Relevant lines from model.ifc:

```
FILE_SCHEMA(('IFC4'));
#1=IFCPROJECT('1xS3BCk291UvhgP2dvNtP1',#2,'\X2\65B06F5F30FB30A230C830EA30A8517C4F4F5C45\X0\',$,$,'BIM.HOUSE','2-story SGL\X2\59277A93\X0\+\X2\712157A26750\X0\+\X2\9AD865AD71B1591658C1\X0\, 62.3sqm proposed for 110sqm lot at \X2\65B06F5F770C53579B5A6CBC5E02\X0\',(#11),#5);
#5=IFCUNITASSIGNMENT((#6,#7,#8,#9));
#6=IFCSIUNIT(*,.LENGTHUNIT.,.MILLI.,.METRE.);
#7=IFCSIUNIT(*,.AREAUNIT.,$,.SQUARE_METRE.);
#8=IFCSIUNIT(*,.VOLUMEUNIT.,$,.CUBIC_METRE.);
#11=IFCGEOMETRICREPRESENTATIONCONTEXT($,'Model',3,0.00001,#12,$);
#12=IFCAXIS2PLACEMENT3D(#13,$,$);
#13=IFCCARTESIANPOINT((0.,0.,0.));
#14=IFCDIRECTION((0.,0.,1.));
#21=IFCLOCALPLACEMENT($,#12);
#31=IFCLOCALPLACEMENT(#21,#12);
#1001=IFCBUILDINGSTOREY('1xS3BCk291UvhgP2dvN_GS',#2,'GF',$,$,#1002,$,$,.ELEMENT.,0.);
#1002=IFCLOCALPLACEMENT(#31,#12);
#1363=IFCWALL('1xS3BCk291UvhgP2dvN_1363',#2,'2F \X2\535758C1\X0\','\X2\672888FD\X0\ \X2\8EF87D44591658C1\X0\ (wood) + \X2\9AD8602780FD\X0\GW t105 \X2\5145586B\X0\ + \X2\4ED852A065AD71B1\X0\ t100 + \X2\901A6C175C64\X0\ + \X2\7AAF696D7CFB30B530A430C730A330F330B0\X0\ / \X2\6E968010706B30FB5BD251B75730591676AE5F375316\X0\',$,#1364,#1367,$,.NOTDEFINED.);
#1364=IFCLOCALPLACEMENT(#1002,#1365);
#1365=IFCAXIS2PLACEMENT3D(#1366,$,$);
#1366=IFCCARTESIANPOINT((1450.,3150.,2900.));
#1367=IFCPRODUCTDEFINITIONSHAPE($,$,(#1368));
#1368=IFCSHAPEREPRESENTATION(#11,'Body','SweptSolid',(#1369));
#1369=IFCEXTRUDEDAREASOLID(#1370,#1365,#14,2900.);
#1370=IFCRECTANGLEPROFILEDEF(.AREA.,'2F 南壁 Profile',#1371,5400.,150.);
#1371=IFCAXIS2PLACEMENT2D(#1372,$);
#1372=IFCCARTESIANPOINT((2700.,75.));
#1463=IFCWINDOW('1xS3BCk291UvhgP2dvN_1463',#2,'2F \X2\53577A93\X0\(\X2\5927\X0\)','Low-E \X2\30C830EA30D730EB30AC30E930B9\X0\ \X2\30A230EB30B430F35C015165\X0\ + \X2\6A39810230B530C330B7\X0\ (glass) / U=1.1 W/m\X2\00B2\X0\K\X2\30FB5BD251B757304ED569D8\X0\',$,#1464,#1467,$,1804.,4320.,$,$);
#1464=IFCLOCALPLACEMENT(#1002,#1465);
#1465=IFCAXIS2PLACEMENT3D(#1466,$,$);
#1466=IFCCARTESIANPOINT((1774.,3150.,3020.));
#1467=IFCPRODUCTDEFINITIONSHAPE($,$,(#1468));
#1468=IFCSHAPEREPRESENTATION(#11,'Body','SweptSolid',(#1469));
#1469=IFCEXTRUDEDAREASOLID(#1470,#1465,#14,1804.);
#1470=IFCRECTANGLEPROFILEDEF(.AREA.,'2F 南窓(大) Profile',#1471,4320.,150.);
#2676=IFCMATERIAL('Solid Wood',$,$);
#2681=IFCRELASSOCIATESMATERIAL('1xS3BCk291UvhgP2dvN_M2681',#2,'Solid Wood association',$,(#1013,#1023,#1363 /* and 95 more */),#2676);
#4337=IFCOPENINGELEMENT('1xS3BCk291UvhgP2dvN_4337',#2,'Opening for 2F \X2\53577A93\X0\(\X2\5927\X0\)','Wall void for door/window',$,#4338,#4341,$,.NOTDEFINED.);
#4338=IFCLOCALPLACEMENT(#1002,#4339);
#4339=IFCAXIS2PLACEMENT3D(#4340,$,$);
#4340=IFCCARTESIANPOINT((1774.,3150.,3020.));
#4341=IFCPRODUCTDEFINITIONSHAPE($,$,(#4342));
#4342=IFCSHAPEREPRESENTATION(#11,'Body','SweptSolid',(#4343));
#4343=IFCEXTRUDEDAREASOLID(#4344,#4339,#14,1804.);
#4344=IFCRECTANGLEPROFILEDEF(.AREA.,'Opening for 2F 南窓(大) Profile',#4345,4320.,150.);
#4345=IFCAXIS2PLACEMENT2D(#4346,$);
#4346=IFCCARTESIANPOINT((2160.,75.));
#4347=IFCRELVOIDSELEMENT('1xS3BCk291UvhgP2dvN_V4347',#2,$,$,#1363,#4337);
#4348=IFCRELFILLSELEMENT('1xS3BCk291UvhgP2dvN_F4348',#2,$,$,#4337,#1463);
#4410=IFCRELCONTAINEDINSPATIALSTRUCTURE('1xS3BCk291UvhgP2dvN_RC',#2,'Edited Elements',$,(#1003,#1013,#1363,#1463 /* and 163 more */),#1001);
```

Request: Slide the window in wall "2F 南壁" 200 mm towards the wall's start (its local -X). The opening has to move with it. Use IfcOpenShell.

```python
import ifcopenshell
import ifcopenshell.api.geometry
import ifcopenshell.util.placement
import ifcopenshell.util.unit

model = ifcopenshell.open("model.ifc")
unit_scale = ifcopenshell.util.unit.calculate_unit_scale(model)

window = model.by_guid("1xS3BCk291UvhgP2dvN_1463")
opening = window.FillsVoids[0].RelatingOpeningElement
wall = opening.VoidsElements[0].RelatingBuildingElement

wall_matrix = ifcopenshell.util.placement.get_local_placement(wall.ObjectPlacement)
shift = wall_matrix[:3, 0] * -0.2 / unit_scale
before = ifcopenshell.util.placement.get_local_placement(window.ObjectPlacement)[:3, 3].copy()

# The window is not placed relative to its opening, so move both.
for product in (opening, window):
    matrix = ifcopenshell.util.placement.get_local_placement(product.ObjectPlacement)
    matrix[:3, 3] += shift
    ifcopenshell.api.geometry.edit_object_placement(model, product=product, matrix=matrix, is_si=False)

after = ifcopenshell.util.placement.get_local_placement(window.ObjectPlacement)[:3, 3]
print("window moved by", (after - before).round(3) + 0.0)

model.write("model_v2.ifc")
```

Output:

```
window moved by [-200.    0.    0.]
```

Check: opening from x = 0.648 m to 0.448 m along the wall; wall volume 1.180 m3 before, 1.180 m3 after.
